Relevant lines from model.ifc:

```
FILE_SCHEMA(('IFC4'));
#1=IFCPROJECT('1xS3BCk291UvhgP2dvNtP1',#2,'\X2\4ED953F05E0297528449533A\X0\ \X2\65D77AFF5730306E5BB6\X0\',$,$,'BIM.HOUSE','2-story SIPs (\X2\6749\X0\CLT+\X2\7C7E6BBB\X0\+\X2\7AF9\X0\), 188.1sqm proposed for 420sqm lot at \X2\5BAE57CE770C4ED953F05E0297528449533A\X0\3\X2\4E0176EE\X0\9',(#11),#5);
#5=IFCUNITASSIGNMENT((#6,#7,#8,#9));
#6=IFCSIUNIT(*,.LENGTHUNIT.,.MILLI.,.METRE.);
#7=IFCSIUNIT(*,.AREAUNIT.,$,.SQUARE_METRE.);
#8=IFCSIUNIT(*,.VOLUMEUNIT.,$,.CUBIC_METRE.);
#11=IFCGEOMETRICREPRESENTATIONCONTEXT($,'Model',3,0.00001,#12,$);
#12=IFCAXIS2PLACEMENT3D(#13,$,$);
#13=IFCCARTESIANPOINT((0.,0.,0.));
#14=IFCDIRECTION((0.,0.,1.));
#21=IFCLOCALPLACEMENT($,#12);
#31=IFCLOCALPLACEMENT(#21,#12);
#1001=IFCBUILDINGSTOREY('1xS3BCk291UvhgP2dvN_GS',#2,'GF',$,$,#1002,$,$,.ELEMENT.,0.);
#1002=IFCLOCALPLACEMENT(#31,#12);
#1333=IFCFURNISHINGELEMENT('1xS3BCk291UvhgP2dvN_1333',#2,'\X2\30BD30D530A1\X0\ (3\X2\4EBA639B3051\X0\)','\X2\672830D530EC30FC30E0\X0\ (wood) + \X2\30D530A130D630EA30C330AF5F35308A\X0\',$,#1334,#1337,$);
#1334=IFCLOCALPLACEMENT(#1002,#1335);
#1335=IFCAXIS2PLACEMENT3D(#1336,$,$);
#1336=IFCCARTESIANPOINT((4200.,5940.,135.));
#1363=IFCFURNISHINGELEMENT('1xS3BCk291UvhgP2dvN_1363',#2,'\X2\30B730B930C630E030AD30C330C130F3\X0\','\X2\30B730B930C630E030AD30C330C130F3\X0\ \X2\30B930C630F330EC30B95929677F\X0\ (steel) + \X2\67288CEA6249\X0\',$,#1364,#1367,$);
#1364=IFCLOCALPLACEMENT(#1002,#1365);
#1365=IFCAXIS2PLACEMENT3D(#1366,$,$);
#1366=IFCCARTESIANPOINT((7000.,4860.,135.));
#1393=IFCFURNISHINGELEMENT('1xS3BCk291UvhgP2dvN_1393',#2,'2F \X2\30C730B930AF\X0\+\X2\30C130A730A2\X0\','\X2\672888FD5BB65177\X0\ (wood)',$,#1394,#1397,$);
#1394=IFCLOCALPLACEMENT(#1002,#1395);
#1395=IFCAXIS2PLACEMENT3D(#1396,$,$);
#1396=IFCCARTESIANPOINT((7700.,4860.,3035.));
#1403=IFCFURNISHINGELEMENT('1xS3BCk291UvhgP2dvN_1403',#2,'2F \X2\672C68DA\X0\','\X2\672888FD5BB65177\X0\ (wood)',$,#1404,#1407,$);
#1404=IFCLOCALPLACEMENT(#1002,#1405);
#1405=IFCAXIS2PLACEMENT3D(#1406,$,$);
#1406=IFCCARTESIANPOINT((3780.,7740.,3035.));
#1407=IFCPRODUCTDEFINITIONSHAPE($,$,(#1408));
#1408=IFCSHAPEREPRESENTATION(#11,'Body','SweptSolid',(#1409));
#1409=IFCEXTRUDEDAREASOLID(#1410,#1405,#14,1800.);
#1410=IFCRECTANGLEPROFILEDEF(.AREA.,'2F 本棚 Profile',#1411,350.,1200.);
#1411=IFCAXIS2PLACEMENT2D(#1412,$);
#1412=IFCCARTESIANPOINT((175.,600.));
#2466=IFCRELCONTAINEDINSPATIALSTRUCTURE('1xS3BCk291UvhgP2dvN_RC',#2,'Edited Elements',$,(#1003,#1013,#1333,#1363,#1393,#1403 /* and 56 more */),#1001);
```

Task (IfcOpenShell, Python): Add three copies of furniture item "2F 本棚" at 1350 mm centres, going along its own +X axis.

```python
import ifcopenshell
import ifcopenshell.api.geometry
import ifcopenshell.api.root
import ifcopenshell.util.element
import ifcopenshell.util.placement
import ifcopenshell.util.unit

model = ifcopenshell.open("model.ifc")
unit_scale = ifcopenshell.util.unit.calculate_unit_scale(model)


def reuse_history(source, copy):
    """copy_class also copies each property set's owner history, people and application; keep the originals."""
    for rel in copy.IsDefinedBy:
        if rel.is_a("IfcRelDefinesByProperties") and (history := rel.RelatingPropertyDefinition.OwnerHistory):
            rel.RelatingPropertyDefinition.OwnerHistory = source.OwnerHistory
            ifcopenshell.util.element.remove_deep2(model, history)


source = model.by_guid("1xS3BCk291UvhgP2dvN_1403")
base = ifcopenshell.util.placement.get_local_placement(source.ObjectPlacement)
step = base[:3, 0] * 1.35 / unit_scale

for i in range(1, 4):
    copy = ifcopenshell.api.root.copy_class(model, product=source)
    copy.Representation = ifcopenshell.util.element.copy_deep(
        model, source.Representation, exclude=["IfcGeometricRepresentationContext", "IfcRepresentationMap"]
    )
    reuse_history(source, copy)
    matrix = base.copy()
    matrix[:3, 3] += i * step
    print("added at", matrix[:3, 3].round(3) + 0.0)
    ifcopenshell.api.geometry.edit_object_placement(model, product=copy, matrix=matrix, is_si=False)

model.write("model_updated.ifc")
```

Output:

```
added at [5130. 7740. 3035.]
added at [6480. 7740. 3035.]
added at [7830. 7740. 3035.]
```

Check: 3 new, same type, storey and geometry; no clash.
